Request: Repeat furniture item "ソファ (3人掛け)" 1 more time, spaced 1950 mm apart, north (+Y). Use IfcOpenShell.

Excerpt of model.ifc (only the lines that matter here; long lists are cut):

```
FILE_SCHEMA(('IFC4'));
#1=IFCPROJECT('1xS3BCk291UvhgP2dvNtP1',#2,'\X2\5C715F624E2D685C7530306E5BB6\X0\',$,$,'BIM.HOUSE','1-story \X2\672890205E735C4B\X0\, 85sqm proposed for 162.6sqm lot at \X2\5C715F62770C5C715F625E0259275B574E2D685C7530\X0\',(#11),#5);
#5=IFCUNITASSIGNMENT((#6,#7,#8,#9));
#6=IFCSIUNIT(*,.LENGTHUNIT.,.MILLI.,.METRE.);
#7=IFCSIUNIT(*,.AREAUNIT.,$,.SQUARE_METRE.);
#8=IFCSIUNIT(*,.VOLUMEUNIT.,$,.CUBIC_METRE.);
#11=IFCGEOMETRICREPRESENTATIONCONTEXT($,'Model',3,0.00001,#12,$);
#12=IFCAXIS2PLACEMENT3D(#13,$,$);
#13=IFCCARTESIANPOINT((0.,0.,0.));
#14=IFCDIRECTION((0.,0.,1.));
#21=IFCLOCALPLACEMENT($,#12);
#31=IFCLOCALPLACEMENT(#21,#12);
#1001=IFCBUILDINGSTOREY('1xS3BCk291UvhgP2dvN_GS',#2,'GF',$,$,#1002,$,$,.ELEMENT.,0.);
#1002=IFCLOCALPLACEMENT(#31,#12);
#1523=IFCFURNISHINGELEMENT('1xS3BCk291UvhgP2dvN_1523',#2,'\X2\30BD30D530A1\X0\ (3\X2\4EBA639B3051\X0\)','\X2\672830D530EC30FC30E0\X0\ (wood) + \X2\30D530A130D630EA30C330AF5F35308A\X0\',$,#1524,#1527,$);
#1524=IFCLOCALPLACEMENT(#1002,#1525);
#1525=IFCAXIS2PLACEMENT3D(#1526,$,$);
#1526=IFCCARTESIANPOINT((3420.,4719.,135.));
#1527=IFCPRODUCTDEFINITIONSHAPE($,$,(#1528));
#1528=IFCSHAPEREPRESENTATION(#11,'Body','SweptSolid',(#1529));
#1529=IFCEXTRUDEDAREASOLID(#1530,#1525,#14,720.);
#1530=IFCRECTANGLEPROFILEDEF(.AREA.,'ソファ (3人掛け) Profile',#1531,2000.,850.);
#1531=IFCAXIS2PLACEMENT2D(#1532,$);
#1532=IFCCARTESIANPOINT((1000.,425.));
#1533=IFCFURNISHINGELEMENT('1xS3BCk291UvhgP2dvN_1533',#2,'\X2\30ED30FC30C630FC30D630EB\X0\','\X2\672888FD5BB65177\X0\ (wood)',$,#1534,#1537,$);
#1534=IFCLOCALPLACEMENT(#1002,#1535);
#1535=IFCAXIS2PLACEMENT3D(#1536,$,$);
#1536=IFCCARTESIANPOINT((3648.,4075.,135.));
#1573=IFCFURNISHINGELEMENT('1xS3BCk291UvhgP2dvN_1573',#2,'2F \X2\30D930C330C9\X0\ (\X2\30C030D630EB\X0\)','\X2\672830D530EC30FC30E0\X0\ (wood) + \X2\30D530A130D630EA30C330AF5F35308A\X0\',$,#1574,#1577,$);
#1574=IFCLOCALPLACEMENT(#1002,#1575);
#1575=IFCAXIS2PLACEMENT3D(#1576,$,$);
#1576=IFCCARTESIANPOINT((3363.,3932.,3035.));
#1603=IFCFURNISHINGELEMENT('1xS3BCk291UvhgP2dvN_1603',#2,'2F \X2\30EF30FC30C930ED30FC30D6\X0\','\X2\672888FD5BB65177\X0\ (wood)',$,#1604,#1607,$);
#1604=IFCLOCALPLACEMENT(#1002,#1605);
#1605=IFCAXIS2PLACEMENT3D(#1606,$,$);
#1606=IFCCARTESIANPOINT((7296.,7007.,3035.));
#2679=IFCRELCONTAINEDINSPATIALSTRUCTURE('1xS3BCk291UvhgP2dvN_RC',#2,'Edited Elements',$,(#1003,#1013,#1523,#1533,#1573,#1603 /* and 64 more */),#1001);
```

```python
import numpy as np
import ifcopenshell
import ifcopenshell.api.geometry
import ifcopenshell.api.root
import ifcopenshell.util.element
import ifcopenshell.util.placement
import ifcopenshell.util.unit

model = ifcopenshell.open("model.ifc")
unit_scale = ifcopenshell.util.unit.calculate_unit_scale(model)


def reuse_history(source, copy):
    """copy_class also copies each property set's owner history, people and application; keep the originals."""
    for rel in copy.IsDefinedBy:
        if rel.is_a("IfcRelDefinesByProperties") and (history := rel.RelatingPropertyDefinition.OwnerHistory):
            rel.RelatingPropertyDefinition.OwnerHistory = source.OwnerHistory
            ifcopenshell.util.element.remove_deep2(model, history)


source = model.by_guid("1xS3BCk291UvhgP2dvN_1523")
base = ifcopenshell.util.placement.get_local_placement(source.ObjectPlacement)
step = np.array([0.0, 1.0, 0.0]) * 1.95 / unit_scale

for i in range(1, 2):
    copy = ifcopenshell.api.root.copy_class(model, product=source)
    copy.Representation = ifcopenshell.util.element.copy_deep(
        model, source.Representation, exclude=["IfcGeometricRepresentationContext", "IfcRepresentationMap"]
    )
    reuse_history(source, copy)
    matrix = base.copy()
    matrix[:3, 3] += i * step
    print("added at", matrix[:3, 3].round(3) + 0.0)
    ifcopenshell.api.geometry.edit_object_placement(model, product=copy, matrix=matrix, is_si=False)

model.write("model_updated.ifc")
```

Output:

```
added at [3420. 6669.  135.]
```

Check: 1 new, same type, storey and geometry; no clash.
